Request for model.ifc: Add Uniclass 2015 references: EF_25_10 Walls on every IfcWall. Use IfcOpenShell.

First a look at what the model holds.

```python
import ifcopenshell

model = ifcopenshell.open("model.ifc")
print(model.schema)
print("classifications:", [c.Name for c in model.by_type("IfcClassification")])
for ifc_class in ("IfcDoor", "IfcRoof", "IfcStair", "IfcWall", "IfcWindow"):
    print(ifc_class, len(model.by_type(ifc_class)))
```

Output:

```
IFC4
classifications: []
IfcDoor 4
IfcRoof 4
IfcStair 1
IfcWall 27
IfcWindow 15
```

```python
import ifcopenshell
import ifcopenshell.api.classification

model = ifcopenshell.open("model.ifc")

system = ifcopenshell.api.classification.add_classification(model, classification="Uniclass 2015")

codes = {
    "IfcWall": ("EF_25_10", "Walls"),
}
for ifc_class, (code, name) in codes.items():
    products = model.by_type(ifc_class)
    ifcopenshell.api.classification.add_reference(
        model, products=products, classification=system, identification=code, name=name
    )
    print(code, len(products))

model.write("model_edited.ifc")
```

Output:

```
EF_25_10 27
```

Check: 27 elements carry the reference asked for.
